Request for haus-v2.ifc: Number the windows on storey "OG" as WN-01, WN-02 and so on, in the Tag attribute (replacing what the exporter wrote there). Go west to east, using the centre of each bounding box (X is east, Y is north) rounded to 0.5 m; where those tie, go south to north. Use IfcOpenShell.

First a look at what the model holds.

```python
import ifcopenshell
import ifcopenshell.util.element
import ifcopenshell.util.placement

model = ifcopenshell.open("haus-v2.ifc")
print(model.schema)
storey = next(s for s in model.by_type("IfcBuildingStorey") if s.Name == "OG")
windows = [e for e in ifcopenshell.util.element.get_decomposition(storey) if e.is_a("IfcWindow")]
for e in sorted(windows, key=lambda e: e.id()):
    origin = ifcopenshell.util.placement.get_local_placement(e.ObjectPlacement)[:3, 3]
    print(e.id(), e.Tag, e.Name, origin.round(2) + 0.0, sep=" | ")
```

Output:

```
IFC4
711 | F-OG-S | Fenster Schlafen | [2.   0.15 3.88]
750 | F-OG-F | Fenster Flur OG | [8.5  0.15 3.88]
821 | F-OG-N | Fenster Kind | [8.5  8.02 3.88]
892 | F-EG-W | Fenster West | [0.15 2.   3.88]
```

```python
import ifcopenshell
import ifcopenshell.geom
import ifcopenshell.util.element
import ifcopenshell.util.shape

model = ifcopenshell.open("haus-v2.ifc")
settings = ifcopenshell.geom.settings()
settings.set("use-world-coords", True)


def centre(element):
    shape = ifcopenshell.geom.create_shape(settings, element)
    return ifcopenshell.util.shape.get_bbox_centroid(shape.geometry)


storey = next(s for s in model.by_type("IfcBuildingStorey") if s.Name == "OG")
windows = [e for e in ifcopenshell.util.element.get_decomposition(storey) if e.is_a("IfcWindow")]

# Insertion points can sit at a corner or the storey origin, so sort by the geometry (in metres).
centres = {e: centre(e) for e in windows}
windows.sort(key=lambda e: (round(centres[e][0] / 0.5), centres[e][1]))

for i, e in enumerate(windows, start=1):
    number = f"WN-{i:02d}"
    e.Tag = number
    print(e.id(), number)

model.write("haus-v2_updated.ifc")
```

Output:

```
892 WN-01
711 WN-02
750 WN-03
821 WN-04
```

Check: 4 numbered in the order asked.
